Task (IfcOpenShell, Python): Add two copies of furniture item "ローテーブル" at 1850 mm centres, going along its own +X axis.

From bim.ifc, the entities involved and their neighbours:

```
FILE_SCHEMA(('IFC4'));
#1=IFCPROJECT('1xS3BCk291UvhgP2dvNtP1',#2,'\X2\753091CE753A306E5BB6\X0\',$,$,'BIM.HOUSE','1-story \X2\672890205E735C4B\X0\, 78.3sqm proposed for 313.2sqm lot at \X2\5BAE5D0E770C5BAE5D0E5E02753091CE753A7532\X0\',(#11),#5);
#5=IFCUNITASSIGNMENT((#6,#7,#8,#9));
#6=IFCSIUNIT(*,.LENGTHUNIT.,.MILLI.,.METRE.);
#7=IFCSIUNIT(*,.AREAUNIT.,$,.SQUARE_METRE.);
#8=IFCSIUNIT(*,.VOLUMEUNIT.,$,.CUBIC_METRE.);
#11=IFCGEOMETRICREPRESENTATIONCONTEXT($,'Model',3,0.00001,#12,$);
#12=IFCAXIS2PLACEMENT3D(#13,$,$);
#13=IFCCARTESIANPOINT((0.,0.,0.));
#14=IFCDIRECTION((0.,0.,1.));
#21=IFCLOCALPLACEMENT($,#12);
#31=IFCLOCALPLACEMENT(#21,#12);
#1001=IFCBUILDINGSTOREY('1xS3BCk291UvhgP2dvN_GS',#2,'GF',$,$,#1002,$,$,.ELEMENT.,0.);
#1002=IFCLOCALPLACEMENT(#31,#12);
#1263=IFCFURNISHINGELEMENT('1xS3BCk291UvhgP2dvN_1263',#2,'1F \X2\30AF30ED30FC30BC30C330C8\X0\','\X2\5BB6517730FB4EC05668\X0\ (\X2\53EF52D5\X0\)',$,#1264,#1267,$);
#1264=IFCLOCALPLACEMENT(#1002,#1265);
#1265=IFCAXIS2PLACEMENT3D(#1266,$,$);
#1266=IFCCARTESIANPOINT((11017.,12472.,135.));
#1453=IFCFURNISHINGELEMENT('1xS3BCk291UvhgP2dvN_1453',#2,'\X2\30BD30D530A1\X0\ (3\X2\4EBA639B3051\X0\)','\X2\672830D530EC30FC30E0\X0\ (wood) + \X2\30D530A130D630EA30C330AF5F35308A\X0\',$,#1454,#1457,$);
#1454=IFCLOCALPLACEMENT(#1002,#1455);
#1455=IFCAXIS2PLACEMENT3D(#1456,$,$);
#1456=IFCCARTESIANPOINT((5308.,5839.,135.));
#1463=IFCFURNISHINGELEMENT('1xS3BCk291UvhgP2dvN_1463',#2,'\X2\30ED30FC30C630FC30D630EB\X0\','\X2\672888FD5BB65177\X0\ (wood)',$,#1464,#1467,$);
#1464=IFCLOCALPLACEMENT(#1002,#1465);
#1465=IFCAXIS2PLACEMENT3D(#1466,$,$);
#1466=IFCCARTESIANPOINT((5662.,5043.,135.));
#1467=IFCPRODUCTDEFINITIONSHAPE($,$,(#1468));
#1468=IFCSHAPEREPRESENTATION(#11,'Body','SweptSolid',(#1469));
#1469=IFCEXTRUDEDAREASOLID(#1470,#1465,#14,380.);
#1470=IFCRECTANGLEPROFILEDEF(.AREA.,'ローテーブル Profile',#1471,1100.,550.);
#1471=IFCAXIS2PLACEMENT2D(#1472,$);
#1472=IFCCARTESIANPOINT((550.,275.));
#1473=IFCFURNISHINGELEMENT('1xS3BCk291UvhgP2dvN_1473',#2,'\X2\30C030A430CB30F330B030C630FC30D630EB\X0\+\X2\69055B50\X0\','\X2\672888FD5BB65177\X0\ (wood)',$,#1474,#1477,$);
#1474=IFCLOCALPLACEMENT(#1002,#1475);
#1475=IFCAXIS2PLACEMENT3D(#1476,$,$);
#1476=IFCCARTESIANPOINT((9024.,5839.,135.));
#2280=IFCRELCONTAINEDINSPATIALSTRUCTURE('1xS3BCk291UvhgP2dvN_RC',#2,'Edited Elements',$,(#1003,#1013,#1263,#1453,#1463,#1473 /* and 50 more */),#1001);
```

```python
import ifcopenshell
import ifcopenshell.api.geometry
import ifcopenshell.api.root
import ifcopenshell.util.element
import ifcopenshell.util.placement
import ifcopenshell.util.unit

model = ifcopenshell.open("bim.ifc")
unit_scale = ifcopenshell.util.unit.calculate_unit_scale(model)


def reuse_history(source, copy):
    """copy_class also copies each property set's owner history, people and application; keep the originals."""
    for rel in copy.IsDefinedBy:
        if rel.is_a("IfcRelDefinesByProperties") and (history := rel.RelatingPropertyDefinition.OwnerHistory):
            rel.RelatingPropertyDefinition.OwnerHistory = source.OwnerHistory
            ifcopenshell.util.element.remove_deep2(model, history)


source = model.by_guid("1xS3BCk291UvhgP2dvN_1463")
base = ifcopenshell.util.placement.get_local_placement(source.ObjectPlacement)
step = base[:3, 0] * 1.85 / unit_scale

for i in range(1, 3):
    copy = ifcopenshell.api.root.copy_class(model, product=source)
    copy.Representation = ifcopenshell.util.element.copy_deep(
        model, source.Representation, exclude=["IfcGeometricRepresentationContext", "IfcRepresentationMap"]
    )
    reuse_history(source, copy)
    matrix = base.copy()
    matrix[:3, 3] += i * step
    print("added at", matrix[:3, 3].round(3) + 0.0)
    ifcopenshell.api.geometry.edit_object_placement(model, product=copy, matrix=matrix, is_si=False)

model.write("bim_edited.ifc")
```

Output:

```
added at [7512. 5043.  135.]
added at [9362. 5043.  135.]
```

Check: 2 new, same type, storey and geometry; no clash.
